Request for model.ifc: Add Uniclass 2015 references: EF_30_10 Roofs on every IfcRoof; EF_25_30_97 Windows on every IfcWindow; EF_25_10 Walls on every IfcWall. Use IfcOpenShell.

First a look at what the model holds.

```python
import ifcopenshell

model = ifcopenshell.open("model.ifc")
print(model.schema)
print("classifications:", [c.Name for c in model.by_type("IfcClassification")])
for ifc_class in ("IfcDoor", "IfcRoof", "IfcStair", "IfcWall", "IfcWindow"):
    print(ifc_class, len(model.by_type(ifc_class)))
```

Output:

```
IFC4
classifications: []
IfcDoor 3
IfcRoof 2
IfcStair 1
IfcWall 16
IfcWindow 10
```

```python
import ifcopenshell
import ifcopenshell.api.classification

model = ifcopenshell.open("model.ifc")

system = ifcopenshell.api.classification.add_classification(model, classification="Uniclass 2015")

codes = {
    "IfcRoof": ("EF_30_10", "Roofs"),
    "IfcWindow": ("EF_25_30_97", "Windows"),
    "IfcWall": ("EF_25_10", "Walls"),
}
for ifc_class, (code, name) in codes.items():
    products = model.by_type(ifc_class)
    ifcopenshell.api.classification.add_reference(
        model, products=products, classification=system, identification=code, name=name
    )
    print(code, len(products))

model.write("model_v2.ifc")
```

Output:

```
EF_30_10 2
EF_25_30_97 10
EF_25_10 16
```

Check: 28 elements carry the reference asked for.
